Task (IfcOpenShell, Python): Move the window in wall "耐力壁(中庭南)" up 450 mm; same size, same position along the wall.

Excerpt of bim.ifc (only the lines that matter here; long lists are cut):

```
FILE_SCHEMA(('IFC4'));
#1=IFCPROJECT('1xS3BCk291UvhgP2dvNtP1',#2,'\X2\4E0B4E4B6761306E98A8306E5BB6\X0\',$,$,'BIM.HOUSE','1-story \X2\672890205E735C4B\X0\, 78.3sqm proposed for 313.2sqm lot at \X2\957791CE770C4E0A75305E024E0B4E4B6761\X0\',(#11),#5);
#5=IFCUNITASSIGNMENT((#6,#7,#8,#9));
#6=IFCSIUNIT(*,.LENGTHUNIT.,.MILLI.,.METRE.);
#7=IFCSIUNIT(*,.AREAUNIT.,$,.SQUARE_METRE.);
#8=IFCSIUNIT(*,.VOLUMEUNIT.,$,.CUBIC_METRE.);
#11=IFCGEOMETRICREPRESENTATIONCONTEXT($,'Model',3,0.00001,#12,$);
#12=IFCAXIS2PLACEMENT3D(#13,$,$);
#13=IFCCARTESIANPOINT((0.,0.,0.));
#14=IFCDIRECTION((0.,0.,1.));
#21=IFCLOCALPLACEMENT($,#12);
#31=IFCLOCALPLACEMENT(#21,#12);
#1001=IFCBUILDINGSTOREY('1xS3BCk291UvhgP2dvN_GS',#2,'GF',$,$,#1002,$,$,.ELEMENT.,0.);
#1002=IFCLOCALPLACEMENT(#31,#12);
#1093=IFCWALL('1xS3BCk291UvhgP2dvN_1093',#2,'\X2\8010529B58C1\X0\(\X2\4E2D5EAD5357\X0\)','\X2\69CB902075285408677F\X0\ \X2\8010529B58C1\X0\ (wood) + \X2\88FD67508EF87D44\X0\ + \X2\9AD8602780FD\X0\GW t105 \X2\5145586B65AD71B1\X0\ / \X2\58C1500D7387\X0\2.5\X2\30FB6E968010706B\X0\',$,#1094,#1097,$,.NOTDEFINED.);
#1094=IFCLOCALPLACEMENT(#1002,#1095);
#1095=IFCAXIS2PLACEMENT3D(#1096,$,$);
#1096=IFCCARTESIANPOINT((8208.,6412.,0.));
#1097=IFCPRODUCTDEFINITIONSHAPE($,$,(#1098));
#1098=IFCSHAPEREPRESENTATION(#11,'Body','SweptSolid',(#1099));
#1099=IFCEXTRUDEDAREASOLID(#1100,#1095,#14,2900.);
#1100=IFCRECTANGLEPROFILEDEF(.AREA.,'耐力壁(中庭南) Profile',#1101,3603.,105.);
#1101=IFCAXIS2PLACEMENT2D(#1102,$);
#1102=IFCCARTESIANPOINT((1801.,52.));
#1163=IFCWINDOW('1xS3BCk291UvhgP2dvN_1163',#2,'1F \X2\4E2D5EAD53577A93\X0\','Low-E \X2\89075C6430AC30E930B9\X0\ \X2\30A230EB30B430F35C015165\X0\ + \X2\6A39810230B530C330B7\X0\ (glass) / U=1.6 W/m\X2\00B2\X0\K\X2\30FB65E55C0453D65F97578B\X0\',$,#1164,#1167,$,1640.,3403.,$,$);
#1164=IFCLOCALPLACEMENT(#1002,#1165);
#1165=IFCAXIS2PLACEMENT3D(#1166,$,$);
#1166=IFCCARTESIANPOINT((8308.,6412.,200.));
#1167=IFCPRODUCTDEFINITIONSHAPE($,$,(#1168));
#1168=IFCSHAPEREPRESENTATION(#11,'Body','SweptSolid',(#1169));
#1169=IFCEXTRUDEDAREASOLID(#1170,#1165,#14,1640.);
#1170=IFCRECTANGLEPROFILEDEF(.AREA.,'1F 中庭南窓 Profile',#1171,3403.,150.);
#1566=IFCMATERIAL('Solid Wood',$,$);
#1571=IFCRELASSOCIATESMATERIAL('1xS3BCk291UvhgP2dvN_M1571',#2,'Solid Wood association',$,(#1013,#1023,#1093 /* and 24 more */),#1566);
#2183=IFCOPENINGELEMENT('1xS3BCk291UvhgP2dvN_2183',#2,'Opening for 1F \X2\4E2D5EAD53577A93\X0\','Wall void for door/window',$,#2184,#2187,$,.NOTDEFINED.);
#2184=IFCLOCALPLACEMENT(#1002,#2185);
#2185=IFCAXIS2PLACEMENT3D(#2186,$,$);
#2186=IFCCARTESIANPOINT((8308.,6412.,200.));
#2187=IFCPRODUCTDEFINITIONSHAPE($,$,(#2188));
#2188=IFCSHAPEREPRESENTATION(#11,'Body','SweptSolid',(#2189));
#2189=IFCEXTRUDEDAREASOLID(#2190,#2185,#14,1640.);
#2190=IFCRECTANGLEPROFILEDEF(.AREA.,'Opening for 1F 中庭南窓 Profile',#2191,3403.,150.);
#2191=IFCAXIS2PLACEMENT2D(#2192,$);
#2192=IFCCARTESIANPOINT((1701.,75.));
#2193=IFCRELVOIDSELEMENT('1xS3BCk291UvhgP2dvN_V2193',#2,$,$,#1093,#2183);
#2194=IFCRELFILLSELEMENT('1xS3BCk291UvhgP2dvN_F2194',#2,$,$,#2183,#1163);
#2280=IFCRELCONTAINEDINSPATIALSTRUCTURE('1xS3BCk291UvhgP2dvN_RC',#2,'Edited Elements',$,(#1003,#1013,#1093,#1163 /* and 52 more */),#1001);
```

```python
import numpy as np
import ifcopenshell
import ifcopenshell.api.geometry
import ifcopenshell.util.placement
import ifcopenshell.util.unit

model = ifcopenshell.open("bim.ifc")
unit_scale = ifcopenshell.util.unit.calculate_unit_scale(model)

window = model.by_guid("1xS3BCk291UvhgP2dvN_1163")
opening = window.FillsVoids[0].RelatingOpeningElement
dz = 0.45 / unit_scale

shift = np.array([0.0, 0.0, dz])
# The window is not placed relative to its opening, so move both.
for product in (opening, window):
    matrix = ifcopenshell.util.placement.get_local_placement(product.ObjectPlacement)
    matrix[:3, 3] += shift
    ifcopenshell.api.geometry.edit_object_placement(model, product=product, matrix=matrix, is_si=False)

print(f"moved by {dz * unit_scale:+.3f} m")

model.write("bim_v2.ifc")
```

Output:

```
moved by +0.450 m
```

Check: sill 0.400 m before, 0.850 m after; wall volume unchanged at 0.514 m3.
